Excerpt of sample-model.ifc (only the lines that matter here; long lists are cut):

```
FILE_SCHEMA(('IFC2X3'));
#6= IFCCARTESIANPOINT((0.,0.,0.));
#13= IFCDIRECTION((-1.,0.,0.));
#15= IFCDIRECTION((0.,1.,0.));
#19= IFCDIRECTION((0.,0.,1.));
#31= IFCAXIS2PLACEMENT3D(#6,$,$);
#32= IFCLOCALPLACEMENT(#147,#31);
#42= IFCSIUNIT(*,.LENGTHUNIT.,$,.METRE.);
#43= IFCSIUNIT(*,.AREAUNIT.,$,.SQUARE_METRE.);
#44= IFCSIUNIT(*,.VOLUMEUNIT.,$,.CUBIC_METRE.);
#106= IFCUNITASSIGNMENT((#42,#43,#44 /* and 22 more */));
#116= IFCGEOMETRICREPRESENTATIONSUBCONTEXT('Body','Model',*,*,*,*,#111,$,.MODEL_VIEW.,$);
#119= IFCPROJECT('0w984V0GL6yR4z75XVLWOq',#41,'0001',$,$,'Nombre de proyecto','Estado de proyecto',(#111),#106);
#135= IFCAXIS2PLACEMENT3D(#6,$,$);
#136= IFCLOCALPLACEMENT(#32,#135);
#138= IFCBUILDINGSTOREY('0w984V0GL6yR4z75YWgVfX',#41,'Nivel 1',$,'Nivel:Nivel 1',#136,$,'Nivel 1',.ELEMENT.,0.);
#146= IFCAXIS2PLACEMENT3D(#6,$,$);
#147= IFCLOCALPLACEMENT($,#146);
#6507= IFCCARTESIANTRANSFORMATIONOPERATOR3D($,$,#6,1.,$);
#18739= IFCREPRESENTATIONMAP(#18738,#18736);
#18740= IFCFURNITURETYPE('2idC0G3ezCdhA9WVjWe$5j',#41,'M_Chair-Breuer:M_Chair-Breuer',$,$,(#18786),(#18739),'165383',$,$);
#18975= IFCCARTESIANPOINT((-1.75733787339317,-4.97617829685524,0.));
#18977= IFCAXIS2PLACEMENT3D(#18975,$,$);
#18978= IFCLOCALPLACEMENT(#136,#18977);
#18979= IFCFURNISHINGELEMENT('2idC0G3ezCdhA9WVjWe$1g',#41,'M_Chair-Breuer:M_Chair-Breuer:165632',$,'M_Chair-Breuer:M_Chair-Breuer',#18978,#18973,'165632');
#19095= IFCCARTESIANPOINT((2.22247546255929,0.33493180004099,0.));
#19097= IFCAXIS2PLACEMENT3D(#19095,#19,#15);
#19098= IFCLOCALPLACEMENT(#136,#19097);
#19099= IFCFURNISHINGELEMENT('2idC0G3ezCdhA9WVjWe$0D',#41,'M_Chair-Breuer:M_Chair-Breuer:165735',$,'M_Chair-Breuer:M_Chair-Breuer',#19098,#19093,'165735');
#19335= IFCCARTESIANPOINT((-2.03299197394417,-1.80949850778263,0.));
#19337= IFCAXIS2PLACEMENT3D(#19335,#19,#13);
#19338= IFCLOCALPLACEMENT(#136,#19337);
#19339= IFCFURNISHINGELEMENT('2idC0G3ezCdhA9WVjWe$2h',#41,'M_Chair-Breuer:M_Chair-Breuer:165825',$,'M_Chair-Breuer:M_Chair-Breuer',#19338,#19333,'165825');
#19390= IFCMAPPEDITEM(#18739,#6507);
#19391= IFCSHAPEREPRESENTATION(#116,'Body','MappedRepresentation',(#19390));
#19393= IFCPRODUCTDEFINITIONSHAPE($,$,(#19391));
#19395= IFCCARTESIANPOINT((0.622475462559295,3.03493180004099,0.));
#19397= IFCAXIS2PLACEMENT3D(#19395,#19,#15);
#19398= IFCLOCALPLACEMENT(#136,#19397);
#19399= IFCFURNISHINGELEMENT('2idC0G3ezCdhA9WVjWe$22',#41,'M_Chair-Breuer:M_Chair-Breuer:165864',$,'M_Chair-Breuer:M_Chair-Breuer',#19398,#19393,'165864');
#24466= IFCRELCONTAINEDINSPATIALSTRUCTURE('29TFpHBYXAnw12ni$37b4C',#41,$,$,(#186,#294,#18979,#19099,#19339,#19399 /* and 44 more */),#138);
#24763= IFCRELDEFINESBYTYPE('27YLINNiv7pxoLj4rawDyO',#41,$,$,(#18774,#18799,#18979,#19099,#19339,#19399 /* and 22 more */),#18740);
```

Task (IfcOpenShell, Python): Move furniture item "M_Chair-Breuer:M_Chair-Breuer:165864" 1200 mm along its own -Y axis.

```python
import ifcopenshell
import ifcopenshell.api.geometry
import ifcopenshell.util.placement

model = ifcopenshell.open("sample-model.ifc")

item = model.by_guid("2idC0G3ezCdhA9WVjWe$22")
matrix = ifcopenshell.util.placement.get_local_placement(item.ObjectPlacement)
matrix[:3, 3] -= matrix[:3, 1] * 1.2
ifcopenshell.api.geometry.edit_object_placement(model, product=item, matrix=matrix, is_si=False)

print(ifcopenshell.util.placement.get_local_placement(item.ObjectPlacement).round(3) + 0.0)

model.write("sample-model_edited.ifc")
```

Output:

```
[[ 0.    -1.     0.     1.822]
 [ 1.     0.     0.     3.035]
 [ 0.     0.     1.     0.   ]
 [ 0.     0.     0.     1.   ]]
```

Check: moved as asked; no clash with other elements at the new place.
